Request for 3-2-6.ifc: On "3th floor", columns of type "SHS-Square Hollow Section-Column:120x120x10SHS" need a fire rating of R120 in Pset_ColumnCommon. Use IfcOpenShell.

First a look at what the model holds.

```python
import ifcopenshell
import ifcopenshell.util.element

model = ifcopenshell.open("3-2-6.ifc")
print(model.schema)
storey = next(s for s in model.by_type("IfcBuildingStorey") if s.Name == "3th floor")
columns = [e for e in ifcopenshell.util.element.get_decomposition(storey) if e.is_a("IfcColumn")]
seen = {}
for e in columns:
    element_type = ifcopenshell.util.element.get_type(e)
    key = (element_type.Name if element_type != e and element_type else None, ifcopenshell.util.element.get_pset(e, "Pset_ColumnCommon", "FireRating"))
    seen[key] = seen.get(key, 0) + 1
for (name, value), count in sorted(seen.items(), key=str):
    print(count, "x", name, "|", value)
```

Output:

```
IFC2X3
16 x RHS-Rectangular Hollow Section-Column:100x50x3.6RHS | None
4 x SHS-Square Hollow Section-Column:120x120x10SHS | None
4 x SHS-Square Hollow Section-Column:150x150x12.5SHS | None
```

```python
import ifcopenshell
import ifcopenshell.api.pset
import ifcopenshell.util.element

model = ifcopenshell.open("3-2-6.ifc")

storey = next(s for s in model.by_type("IfcBuildingStorey") if s.Name == "3th floor")
columns = [e for e in ifcopenshell.util.element.get_decomposition(storey) if e.is_a("IfcColumn")]

count = 0
for e in columns:
    element_type = ifcopenshell.util.element.get_type(e)
    if element_type in (None, e) or element_type.Name != "SHS-Square Hollow Section-Column:120x120x10SHS":
        continue
    # add_pset returns the element's existing set when there is one.
    pset = ifcopenshell.api.pset.add_pset(model, product=e, name="Pset_ColumnCommon")
    ifcopenshell.api.pset.edit_pset(model, pset=pset, properties={"FireRating": "R120"})
    count += 1

print(count, "columns updated")

model.write("3-2-6-out.ifc")
```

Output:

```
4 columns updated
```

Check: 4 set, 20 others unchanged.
